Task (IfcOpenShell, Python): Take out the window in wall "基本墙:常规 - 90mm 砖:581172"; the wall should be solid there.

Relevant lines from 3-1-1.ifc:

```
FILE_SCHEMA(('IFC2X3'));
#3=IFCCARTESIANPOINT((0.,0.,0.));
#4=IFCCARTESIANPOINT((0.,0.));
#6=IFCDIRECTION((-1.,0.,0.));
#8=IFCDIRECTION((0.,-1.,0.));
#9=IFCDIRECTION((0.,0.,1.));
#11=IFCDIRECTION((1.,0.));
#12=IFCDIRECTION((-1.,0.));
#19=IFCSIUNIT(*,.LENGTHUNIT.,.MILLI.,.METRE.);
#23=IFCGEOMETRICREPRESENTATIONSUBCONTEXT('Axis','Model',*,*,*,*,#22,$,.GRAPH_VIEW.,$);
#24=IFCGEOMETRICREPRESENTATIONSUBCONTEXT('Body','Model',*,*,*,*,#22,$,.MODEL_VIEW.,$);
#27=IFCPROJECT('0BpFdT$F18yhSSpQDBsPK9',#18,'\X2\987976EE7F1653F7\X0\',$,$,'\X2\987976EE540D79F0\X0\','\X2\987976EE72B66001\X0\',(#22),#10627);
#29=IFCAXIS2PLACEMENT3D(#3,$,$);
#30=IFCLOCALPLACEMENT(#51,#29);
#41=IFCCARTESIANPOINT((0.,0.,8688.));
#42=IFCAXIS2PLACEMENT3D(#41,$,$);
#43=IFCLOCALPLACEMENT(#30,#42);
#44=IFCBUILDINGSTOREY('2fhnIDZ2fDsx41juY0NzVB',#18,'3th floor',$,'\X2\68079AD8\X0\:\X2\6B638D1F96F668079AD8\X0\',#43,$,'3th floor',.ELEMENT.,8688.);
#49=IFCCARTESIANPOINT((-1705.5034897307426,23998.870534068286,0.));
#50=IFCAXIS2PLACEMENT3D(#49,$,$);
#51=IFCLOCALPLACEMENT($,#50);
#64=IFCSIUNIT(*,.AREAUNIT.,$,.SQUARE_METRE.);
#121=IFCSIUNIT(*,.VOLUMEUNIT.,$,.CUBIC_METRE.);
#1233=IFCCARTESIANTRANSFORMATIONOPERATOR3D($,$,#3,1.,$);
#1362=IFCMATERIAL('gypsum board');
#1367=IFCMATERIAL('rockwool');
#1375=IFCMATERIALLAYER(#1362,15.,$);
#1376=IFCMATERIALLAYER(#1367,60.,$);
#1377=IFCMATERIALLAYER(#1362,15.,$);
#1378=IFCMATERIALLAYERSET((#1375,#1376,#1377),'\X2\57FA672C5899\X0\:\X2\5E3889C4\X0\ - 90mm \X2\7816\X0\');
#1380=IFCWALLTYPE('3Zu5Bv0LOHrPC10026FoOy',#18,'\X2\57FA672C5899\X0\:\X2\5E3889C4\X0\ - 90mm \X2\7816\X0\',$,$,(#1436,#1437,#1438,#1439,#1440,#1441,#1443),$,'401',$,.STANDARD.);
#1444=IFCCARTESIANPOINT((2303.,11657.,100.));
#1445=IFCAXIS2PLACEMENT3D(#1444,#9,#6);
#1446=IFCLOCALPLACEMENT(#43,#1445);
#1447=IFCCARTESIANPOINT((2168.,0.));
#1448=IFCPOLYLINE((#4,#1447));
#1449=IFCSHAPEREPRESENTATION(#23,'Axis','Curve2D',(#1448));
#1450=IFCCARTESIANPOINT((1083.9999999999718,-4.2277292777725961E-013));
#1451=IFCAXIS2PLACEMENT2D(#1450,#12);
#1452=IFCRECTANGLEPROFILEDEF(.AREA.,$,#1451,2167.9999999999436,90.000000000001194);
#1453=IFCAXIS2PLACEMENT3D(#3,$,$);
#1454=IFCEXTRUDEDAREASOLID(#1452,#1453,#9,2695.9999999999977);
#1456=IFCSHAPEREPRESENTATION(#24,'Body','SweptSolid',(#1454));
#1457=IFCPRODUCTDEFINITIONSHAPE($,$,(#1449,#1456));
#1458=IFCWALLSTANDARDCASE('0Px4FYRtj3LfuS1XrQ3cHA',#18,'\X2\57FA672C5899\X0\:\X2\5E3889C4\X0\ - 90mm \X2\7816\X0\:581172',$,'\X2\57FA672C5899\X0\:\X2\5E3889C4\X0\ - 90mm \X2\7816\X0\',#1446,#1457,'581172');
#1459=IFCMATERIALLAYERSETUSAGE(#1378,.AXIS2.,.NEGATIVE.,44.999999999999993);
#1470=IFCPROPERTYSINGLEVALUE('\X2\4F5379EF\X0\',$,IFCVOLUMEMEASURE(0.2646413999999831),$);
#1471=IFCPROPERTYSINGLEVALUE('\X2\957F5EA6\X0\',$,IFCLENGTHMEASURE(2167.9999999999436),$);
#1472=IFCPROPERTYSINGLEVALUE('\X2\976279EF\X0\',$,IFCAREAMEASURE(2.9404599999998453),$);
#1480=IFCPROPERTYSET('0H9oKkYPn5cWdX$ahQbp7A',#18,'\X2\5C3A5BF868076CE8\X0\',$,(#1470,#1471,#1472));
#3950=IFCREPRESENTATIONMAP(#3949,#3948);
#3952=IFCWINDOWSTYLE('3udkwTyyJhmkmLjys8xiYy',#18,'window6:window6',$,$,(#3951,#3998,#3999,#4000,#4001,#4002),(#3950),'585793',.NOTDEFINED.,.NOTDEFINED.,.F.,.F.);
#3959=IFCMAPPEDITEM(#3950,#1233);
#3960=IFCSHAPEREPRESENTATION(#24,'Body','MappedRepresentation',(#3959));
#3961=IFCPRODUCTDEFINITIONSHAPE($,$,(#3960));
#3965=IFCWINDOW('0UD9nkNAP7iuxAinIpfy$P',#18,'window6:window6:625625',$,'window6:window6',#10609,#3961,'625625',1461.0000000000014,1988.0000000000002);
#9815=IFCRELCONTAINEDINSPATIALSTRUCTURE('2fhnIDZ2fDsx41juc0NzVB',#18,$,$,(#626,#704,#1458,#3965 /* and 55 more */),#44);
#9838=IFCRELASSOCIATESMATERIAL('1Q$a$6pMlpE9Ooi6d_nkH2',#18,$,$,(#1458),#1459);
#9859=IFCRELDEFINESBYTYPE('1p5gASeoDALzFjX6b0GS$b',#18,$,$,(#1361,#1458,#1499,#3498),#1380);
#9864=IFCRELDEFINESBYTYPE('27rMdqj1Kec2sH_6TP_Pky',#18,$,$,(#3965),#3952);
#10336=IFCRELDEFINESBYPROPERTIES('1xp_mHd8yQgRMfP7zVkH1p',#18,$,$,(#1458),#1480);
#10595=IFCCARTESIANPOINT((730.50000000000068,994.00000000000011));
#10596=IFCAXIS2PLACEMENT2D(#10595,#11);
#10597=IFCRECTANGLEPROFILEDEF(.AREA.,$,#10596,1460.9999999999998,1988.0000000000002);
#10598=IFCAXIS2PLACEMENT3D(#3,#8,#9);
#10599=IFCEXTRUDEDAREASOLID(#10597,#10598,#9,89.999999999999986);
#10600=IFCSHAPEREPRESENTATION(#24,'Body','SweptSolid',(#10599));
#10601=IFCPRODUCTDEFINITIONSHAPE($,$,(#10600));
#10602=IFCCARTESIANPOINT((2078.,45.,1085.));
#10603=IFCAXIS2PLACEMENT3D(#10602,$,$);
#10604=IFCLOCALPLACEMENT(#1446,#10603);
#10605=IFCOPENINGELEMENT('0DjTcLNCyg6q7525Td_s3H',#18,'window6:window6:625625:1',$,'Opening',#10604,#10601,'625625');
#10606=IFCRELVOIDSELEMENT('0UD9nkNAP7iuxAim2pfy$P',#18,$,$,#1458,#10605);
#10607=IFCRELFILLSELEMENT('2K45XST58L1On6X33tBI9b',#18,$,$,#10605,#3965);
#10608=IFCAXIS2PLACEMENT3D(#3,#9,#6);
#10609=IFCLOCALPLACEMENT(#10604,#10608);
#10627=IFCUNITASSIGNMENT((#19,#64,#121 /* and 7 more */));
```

```python
import ifcopenshell
import ifcopenshell.api.feature
import ifcopenshell.api.pset
import ifcopenshell.api.root
import ifcopenshell.geom
import ifcopenshell.util.element
import ifcopenshell.util.shape
import ifcopenshell.util.unit

model = ifcopenshell.open("3-1-1.ifc")
area_scale = ifcopenshell.util.unit.calculate_unit_scale(model, "AREAUNIT")
volume_scale = ifcopenshell.util.unit.calculate_unit_scale(model, "VOLUMEUNIT")
settings = ifcopenshell.geom.settings()


def volume(element):
    """Net volume in cubic metres, openings subtracted."""
    shape = ifcopenshell.geom.create_shape(settings, element)
    return ifcopenshell.util.shape.get_volume(shape.geometry)


window = model.by_guid("0UD9nkNAP7iuxAinIpfy$P")
opening = window.FillsVoids[0].RelatingOpeningElement
wall = opening.VoidsElements[0].RelatingBuildingElement
before = volume(wall)

ifcopenshell.api.root.remove_product(model, product=window)
ifcopenshell.api.feature.remove_feature(model, feature=opening)

after = volume(wall)
thickness = 0.09  # wall thickness in metres

# Update the wall's stored quantities.
pset = model.by_id(ifcopenshell.util.element.get_pset(wall, "尺寸标注", should_inherit=False)["id"])
ifcopenshell.api.pset.edit_pset(model, pset=pset, properties={
    "体积": model.create_entity("IfcVolumeMeasure", after / volume_scale),
    "面积": model.create_entity("IfcAreaMeasure", after / thickness / area_scale),
})

print(f"wall volume {before:.3f} -> {after:.3f} m3")

model.write("3-1-1_edited.ifc")
```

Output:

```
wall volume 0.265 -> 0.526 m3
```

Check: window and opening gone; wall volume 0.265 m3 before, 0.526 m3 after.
